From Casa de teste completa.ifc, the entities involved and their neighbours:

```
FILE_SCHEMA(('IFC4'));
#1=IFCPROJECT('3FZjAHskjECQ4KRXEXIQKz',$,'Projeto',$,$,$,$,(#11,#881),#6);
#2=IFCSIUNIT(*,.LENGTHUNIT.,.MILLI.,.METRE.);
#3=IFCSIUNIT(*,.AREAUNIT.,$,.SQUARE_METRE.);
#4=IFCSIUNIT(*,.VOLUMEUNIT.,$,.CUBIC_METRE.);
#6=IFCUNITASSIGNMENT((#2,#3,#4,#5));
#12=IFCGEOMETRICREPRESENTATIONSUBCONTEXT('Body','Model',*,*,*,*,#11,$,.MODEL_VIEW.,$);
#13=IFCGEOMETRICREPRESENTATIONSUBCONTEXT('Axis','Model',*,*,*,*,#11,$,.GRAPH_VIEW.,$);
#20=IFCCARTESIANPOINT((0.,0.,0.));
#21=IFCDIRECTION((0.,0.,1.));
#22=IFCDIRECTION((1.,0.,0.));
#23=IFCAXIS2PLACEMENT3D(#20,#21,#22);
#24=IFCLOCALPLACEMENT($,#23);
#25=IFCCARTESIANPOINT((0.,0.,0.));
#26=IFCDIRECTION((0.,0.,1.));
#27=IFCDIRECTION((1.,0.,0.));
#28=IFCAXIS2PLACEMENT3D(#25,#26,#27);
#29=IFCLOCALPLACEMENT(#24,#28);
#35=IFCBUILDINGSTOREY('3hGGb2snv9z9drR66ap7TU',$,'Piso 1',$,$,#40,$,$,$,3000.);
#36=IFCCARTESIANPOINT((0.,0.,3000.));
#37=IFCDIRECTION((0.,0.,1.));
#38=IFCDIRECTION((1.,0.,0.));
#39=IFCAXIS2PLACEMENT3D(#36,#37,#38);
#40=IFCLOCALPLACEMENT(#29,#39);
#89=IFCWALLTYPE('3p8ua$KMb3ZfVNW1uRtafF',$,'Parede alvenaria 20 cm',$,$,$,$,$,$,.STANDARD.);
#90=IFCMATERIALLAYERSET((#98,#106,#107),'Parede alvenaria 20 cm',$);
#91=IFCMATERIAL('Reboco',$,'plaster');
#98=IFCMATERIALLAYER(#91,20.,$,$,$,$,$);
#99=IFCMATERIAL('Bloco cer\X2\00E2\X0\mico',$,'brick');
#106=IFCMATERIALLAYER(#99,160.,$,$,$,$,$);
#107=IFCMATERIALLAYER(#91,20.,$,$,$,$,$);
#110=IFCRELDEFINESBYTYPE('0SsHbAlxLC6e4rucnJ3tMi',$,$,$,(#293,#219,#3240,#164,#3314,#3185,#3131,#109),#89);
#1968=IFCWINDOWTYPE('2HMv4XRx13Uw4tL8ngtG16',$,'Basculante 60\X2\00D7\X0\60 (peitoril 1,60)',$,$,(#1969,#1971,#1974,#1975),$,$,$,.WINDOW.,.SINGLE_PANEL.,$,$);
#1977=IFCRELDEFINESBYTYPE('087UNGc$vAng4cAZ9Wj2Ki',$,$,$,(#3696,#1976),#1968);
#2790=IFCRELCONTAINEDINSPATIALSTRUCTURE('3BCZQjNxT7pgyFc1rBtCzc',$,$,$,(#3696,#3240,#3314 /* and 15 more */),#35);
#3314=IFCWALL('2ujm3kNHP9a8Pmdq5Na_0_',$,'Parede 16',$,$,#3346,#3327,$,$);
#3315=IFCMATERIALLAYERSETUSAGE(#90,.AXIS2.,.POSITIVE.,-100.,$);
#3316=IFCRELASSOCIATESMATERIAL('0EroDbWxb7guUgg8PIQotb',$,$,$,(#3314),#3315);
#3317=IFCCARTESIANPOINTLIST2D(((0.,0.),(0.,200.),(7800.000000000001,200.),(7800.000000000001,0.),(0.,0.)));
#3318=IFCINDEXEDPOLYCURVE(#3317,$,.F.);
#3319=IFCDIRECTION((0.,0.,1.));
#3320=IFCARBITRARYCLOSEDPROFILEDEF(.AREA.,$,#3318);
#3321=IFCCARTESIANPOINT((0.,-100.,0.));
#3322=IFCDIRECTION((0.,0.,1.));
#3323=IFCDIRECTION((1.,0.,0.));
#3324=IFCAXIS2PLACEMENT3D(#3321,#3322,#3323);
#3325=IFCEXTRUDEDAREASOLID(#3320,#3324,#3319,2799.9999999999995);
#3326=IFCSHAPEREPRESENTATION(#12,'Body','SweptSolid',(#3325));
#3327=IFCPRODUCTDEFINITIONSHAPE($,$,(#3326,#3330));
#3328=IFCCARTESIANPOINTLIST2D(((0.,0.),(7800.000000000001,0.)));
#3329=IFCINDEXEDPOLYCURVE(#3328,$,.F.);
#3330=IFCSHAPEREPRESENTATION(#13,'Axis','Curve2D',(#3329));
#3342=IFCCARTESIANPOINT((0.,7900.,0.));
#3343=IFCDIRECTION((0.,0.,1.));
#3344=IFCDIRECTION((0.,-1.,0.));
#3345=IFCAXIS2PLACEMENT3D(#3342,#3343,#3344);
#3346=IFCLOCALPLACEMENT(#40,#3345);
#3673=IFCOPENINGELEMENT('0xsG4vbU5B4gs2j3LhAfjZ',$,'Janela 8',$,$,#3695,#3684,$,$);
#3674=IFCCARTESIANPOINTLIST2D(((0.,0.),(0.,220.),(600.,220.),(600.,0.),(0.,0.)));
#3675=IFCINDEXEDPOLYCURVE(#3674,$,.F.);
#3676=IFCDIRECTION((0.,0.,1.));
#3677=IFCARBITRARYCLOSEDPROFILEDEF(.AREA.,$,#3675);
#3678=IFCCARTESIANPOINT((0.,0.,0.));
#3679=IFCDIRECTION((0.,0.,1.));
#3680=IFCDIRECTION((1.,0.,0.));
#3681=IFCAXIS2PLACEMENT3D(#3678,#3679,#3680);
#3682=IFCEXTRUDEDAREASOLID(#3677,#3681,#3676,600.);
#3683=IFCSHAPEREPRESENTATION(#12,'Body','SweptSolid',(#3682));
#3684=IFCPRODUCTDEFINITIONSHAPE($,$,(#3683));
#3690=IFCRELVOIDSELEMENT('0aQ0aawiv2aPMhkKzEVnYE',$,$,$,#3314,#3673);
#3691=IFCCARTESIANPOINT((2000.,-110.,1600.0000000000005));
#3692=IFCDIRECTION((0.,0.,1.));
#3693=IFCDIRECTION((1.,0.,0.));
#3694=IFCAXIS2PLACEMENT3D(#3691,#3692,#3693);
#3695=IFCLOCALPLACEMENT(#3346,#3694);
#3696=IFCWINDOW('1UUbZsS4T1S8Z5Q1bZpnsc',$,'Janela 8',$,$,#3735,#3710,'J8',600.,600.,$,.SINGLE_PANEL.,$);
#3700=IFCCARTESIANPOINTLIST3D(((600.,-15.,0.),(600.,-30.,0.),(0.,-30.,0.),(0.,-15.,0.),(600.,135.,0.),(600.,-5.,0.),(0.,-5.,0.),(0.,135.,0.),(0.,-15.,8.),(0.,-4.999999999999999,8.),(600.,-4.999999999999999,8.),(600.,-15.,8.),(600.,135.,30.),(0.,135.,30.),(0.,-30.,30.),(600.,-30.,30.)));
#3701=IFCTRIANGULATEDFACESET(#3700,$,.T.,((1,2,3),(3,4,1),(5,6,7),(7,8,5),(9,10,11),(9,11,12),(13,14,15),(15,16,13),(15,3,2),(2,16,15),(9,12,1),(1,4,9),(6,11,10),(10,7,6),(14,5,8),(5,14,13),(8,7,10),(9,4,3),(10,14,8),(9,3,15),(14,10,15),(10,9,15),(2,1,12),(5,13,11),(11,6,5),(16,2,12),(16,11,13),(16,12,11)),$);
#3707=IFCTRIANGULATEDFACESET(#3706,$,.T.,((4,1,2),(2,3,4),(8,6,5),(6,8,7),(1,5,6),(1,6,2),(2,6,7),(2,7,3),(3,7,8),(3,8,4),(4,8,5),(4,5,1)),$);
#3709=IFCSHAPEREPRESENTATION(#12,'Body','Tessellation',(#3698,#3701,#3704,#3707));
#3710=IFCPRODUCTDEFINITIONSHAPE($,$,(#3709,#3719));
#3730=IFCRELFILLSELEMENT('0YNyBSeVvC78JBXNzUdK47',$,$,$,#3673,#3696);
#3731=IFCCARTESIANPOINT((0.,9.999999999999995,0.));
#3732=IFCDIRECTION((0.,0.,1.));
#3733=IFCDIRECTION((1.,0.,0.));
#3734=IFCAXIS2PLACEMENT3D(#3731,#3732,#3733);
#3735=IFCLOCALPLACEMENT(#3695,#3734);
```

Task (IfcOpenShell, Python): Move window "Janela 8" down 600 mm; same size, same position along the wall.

```python
import numpy as np
import ifcopenshell
import ifcopenshell.api.geometry
import ifcopenshell.util.placement
import ifcopenshell.util.unit

model = ifcopenshell.open("Casa de teste completa.ifc")
unit_scale = ifcopenshell.util.unit.calculate_unit_scale(model)

window = model.by_guid("1UUbZsS4T1S8Z5Q1bZpnsc")
opening = window.FillsVoids[0].RelatingOpeningElement
dz = -0.6 / unit_scale

shift = np.array([0.0, 0.0, dz])
# The window is placed relative to its opening, so it follows when the opening moves.
matrix = ifcopenshell.util.placement.get_local_placement(opening.ObjectPlacement)
matrix[:3, 3] += shift
ifcopenshell.api.geometry.edit_object_placement(
    model, product=opening, matrix=matrix, is_si=False, should_transform_children=True
)

print(f"moved by {dz * unit_scale:+.3f} m")

model.write("Casa de teste completa_updated.ifc")
```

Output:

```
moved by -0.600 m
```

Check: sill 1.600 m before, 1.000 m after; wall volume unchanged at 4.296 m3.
